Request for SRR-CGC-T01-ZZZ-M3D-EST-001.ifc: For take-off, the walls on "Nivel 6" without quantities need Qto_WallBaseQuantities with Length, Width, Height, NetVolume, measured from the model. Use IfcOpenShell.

First a look at what the model holds.

```python
import ifcopenshell
import ifcopenshell.util.element
import ifcopenshell.util.unit

model = ifcopenshell.open("SRR-CGC-T01-ZZZ-M3D-EST-001.ifc")
print(model.schema)
for unit_type in ("LENGTHUNIT", "AREAUNIT", "VOLUMEUNIT"):
    print(unit_type, ifcopenshell.util.unit.calculate_unit_scale(model, unit_type))
storey = next(s for s in model.by_type("IfcBuildingStorey") if s.Name == "Nivel 6")
walls = [e for e in ifcopenshell.util.element.get_decomposition(storey) if e.is_a("IfcWall")]
for e in sorted(walls, key=lambda e: e.id()):
    print(e.id(), e.is_a(), e.Name, list(ifcopenshell.util.element.get_psets(e, qtos_only=True)), sep=" | ")
```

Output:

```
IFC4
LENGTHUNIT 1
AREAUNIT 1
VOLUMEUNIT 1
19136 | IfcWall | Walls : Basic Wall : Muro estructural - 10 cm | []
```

```python
import ifcopenshell
import ifcopenshell.api.pset
import ifcopenshell.geom
import ifcopenshell.util.element
import ifcopenshell.util.shape
import ifcopenshell.util.unit

model = ifcopenshell.open("SRR-CGC-T01-ZZZ-M3D-EST-001.ifc")
unit_scale = ifcopenshell.util.unit.calculate_unit_scale(model)
volume_scale = ifcopenshell.util.unit.calculate_unit_scale(model, "VOLUMEUNIT")
settings = ifcopenshell.geom.settings()

storey = next(s for s in model.by_type("IfcBuildingStorey") if s.Name == "Nivel 6")
walls = [e for e in ifcopenshell.util.element.get_decomposition(storey) if e.is_a("IfcWall")]

for e in sorted(walls, key=lambda e: e.id()):
    if ifcopenshell.util.element.get_psets(e, qtos_only=True, should_inherit=False):
        continue
    # Geometry comes back in metres, in the element's own axes.
    shape = ifcopenshell.geom.create_shape(settings, e)
    values = {
        "Length": ifcopenshell.util.shape.get_x(shape.geometry) / unit_scale,
        "Width": ifcopenshell.util.shape.get_y(shape.geometry) / unit_scale,
        "Height": ifcopenshell.util.shape.get_z(shape.geometry) / unit_scale,
        "NetVolume": ifcopenshell.util.shape.get_volume(shape.geometry) / volume_scale,
    }
    qto = ifcopenshell.api.pset.add_qto(model, product=e, name="Qto_WallBaseQuantities")
    ifcopenshell.api.pset.edit_qto(model, qto=qto, properties=values)
    print(e.id(), {k: round(v, 3) for k, v in values.items()})

model.write("SRR-CGC-T01-ZZZ-M3D-EST-001_v2.ifc")
```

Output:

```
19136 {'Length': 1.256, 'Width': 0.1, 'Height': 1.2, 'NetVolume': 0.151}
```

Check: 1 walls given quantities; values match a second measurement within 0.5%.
